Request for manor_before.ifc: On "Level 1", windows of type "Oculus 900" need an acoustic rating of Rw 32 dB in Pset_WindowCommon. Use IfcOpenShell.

First a look at what the model holds.

```python
import ifcopenshell
import ifcopenshell.util.element

model = ifcopenshell.open("manor_before.ifc")
print(model.schema)
storey = next(s for s in model.by_type("IfcBuildingStorey") if s.Name == "Level 1")
windows = [e for e in ifcopenshell.util.element.get_decomposition(storey) if e.is_a("IfcWindow")]
seen = {}
for e in windows:
    element_type = ifcopenshell.util.element.get_type(e)
    key = (element_type.Name if element_type != e and element_type else None, ifcopenshell.util.element.get_pset(e, "Pset_WindowCommon", "AcousticRating"))
    seen[key] = seen.get(key, 0) + 1
for (name, value), count in sorted(seen.items(), key=str):
    print(count, "x", name, "|", value)
```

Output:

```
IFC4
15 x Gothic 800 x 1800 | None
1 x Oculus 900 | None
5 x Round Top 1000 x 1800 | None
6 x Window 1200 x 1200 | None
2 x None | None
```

```python
import ifcopenshell
import ifcopenshell.api.pset
import ifcopenshell.util.element

model = ifcopenshell.open("manor_before.ifc")

storey = next(s for s in model.by_type("IfcBuildingStorey") if s.Name == "Level 1")
windows = [e for e in ifcopenshell.util.element.get_decomposition(storey) if e.is_a("IfcWindow")]

count = 0
for e in windows:
    element_type = ifcopenshell.util.element.get_type(e)
    if element_type in (None, e) or element_type.Name != "Oculus 900":
        continue
    # add_pset returns the element's existing set when there is one.
    pset = ifcopenshell.api.pset.add_pset(model, product=e, name="Pset_WindowCommon")
    ifcopenshell.api.pset.edit_pset(model, pset=pset, properties={"AcousticRating": "Rw 32 dB"})
    count += 1

print(count, "windows updated")

model.write("manor_before_edited.ifc")
```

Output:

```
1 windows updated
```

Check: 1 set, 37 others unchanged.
